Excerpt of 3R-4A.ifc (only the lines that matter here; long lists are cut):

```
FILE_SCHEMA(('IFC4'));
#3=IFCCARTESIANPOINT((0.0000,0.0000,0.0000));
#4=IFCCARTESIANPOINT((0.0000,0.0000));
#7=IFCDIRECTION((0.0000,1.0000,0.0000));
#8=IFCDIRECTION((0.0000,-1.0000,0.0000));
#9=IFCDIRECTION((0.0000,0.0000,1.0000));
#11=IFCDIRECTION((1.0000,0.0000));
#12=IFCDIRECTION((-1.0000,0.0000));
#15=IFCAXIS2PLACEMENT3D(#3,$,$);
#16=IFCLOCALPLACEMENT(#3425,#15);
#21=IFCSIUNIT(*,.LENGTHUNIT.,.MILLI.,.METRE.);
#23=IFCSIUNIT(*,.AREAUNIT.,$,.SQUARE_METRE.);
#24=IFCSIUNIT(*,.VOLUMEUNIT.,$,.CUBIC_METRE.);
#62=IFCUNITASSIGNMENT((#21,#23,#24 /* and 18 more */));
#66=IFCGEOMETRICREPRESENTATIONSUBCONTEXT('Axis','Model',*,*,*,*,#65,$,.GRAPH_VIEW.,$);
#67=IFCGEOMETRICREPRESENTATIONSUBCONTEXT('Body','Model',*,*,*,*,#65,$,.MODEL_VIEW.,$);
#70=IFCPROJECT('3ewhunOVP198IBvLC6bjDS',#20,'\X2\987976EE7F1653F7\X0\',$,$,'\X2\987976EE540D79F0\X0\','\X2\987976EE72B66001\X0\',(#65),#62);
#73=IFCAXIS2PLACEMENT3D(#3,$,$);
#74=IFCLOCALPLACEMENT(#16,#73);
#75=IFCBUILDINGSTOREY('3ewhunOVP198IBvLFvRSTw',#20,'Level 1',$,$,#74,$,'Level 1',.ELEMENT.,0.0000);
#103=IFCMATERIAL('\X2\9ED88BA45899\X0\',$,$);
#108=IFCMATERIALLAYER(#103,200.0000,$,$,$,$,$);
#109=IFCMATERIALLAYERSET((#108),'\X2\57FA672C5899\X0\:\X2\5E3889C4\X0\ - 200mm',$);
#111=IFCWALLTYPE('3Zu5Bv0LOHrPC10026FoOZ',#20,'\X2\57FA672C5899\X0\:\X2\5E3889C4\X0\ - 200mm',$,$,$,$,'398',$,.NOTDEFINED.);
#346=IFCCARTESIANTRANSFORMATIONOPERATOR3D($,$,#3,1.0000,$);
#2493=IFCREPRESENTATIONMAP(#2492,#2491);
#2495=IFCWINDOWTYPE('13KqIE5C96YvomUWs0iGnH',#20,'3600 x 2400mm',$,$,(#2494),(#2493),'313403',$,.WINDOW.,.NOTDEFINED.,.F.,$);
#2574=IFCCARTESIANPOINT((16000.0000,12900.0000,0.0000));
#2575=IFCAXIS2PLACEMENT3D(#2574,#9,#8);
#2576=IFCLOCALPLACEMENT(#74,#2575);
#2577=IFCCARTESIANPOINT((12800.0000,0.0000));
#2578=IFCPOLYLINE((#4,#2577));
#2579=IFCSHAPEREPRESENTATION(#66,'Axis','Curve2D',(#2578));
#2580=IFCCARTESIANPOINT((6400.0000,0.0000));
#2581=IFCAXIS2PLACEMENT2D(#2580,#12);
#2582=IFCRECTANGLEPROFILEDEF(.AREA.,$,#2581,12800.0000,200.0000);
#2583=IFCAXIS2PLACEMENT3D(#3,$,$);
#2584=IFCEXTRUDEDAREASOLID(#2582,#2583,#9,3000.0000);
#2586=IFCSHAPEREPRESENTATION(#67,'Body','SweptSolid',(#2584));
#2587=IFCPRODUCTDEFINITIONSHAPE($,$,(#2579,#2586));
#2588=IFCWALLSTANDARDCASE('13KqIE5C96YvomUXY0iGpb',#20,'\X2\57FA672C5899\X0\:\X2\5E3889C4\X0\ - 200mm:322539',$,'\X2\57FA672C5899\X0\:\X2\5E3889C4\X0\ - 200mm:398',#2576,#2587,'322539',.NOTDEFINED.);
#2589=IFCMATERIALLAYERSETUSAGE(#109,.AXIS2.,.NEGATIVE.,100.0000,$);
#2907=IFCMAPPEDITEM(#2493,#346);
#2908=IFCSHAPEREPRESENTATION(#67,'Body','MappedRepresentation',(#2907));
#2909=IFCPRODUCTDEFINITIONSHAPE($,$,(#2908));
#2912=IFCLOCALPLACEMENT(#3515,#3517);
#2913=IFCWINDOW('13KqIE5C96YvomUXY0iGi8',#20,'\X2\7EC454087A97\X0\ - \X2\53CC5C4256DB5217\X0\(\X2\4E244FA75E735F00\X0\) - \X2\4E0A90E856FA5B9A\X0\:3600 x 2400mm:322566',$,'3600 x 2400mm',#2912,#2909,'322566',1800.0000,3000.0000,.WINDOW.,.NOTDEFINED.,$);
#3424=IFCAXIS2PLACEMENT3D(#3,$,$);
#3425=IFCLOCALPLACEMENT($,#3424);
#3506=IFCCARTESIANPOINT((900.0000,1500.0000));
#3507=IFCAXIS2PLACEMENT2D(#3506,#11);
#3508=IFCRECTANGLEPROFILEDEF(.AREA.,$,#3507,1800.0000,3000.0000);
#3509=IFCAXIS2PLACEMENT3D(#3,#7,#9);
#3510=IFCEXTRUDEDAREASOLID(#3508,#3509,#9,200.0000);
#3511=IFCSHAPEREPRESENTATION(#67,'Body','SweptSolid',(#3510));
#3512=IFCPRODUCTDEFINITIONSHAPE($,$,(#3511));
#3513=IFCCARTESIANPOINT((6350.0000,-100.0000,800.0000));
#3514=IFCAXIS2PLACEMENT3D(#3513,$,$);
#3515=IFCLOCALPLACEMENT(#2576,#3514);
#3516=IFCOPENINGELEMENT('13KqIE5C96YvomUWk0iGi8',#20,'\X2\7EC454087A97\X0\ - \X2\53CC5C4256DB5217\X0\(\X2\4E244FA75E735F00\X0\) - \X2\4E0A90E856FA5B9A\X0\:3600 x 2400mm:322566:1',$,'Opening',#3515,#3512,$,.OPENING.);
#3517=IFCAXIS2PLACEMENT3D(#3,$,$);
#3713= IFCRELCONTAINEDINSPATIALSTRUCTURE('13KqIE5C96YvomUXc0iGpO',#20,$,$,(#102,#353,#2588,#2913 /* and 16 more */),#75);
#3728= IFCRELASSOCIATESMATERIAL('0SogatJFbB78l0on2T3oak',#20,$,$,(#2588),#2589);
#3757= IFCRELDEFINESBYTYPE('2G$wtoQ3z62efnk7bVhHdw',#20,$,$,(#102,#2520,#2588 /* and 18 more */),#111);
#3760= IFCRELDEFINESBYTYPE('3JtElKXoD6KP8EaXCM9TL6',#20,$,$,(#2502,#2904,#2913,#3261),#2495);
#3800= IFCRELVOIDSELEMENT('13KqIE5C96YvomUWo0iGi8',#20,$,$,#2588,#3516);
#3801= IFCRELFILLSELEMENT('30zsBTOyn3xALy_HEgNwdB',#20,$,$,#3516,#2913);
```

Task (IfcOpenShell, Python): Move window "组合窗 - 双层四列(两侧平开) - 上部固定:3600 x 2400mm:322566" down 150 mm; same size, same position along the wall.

```python
import numpy as np
import ifcopenshell
import ifcopenshell.api.geometry
import ifcopenshell.util.placement
import ifcopenshell.util.unit

model = ifcopenshell.open("3R-4A.ifc")
unit_scale = ifcopenshell.util.unit.calculate_unit_scale(model)

window = model.by_guid("13KqIE5C96YvomUXY0iGi8")
opening = window.FillsVoids[0].RelatingOpeningElement
dz = -0.15 / unit_scale

shift = np.array([0.0, 0.0, dz])
# The window is placed relative to its opening, so it follows when the opening moves.
matrix = ifcopenshell.util.placement.get_local_placement(opening.ObjectPlacement)
matrix[:3, 3] += shift
ifcopenshell.api.geometry.edit_object_placement(
    model, product=opening, matrix=matrix, is_si=False, should_transform_children=True
)

print(f"moved by {dz * unit_scale:+.3f} m")

model.write("3R-4A-out.ifc")
```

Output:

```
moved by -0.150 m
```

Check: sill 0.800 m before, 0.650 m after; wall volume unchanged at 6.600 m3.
